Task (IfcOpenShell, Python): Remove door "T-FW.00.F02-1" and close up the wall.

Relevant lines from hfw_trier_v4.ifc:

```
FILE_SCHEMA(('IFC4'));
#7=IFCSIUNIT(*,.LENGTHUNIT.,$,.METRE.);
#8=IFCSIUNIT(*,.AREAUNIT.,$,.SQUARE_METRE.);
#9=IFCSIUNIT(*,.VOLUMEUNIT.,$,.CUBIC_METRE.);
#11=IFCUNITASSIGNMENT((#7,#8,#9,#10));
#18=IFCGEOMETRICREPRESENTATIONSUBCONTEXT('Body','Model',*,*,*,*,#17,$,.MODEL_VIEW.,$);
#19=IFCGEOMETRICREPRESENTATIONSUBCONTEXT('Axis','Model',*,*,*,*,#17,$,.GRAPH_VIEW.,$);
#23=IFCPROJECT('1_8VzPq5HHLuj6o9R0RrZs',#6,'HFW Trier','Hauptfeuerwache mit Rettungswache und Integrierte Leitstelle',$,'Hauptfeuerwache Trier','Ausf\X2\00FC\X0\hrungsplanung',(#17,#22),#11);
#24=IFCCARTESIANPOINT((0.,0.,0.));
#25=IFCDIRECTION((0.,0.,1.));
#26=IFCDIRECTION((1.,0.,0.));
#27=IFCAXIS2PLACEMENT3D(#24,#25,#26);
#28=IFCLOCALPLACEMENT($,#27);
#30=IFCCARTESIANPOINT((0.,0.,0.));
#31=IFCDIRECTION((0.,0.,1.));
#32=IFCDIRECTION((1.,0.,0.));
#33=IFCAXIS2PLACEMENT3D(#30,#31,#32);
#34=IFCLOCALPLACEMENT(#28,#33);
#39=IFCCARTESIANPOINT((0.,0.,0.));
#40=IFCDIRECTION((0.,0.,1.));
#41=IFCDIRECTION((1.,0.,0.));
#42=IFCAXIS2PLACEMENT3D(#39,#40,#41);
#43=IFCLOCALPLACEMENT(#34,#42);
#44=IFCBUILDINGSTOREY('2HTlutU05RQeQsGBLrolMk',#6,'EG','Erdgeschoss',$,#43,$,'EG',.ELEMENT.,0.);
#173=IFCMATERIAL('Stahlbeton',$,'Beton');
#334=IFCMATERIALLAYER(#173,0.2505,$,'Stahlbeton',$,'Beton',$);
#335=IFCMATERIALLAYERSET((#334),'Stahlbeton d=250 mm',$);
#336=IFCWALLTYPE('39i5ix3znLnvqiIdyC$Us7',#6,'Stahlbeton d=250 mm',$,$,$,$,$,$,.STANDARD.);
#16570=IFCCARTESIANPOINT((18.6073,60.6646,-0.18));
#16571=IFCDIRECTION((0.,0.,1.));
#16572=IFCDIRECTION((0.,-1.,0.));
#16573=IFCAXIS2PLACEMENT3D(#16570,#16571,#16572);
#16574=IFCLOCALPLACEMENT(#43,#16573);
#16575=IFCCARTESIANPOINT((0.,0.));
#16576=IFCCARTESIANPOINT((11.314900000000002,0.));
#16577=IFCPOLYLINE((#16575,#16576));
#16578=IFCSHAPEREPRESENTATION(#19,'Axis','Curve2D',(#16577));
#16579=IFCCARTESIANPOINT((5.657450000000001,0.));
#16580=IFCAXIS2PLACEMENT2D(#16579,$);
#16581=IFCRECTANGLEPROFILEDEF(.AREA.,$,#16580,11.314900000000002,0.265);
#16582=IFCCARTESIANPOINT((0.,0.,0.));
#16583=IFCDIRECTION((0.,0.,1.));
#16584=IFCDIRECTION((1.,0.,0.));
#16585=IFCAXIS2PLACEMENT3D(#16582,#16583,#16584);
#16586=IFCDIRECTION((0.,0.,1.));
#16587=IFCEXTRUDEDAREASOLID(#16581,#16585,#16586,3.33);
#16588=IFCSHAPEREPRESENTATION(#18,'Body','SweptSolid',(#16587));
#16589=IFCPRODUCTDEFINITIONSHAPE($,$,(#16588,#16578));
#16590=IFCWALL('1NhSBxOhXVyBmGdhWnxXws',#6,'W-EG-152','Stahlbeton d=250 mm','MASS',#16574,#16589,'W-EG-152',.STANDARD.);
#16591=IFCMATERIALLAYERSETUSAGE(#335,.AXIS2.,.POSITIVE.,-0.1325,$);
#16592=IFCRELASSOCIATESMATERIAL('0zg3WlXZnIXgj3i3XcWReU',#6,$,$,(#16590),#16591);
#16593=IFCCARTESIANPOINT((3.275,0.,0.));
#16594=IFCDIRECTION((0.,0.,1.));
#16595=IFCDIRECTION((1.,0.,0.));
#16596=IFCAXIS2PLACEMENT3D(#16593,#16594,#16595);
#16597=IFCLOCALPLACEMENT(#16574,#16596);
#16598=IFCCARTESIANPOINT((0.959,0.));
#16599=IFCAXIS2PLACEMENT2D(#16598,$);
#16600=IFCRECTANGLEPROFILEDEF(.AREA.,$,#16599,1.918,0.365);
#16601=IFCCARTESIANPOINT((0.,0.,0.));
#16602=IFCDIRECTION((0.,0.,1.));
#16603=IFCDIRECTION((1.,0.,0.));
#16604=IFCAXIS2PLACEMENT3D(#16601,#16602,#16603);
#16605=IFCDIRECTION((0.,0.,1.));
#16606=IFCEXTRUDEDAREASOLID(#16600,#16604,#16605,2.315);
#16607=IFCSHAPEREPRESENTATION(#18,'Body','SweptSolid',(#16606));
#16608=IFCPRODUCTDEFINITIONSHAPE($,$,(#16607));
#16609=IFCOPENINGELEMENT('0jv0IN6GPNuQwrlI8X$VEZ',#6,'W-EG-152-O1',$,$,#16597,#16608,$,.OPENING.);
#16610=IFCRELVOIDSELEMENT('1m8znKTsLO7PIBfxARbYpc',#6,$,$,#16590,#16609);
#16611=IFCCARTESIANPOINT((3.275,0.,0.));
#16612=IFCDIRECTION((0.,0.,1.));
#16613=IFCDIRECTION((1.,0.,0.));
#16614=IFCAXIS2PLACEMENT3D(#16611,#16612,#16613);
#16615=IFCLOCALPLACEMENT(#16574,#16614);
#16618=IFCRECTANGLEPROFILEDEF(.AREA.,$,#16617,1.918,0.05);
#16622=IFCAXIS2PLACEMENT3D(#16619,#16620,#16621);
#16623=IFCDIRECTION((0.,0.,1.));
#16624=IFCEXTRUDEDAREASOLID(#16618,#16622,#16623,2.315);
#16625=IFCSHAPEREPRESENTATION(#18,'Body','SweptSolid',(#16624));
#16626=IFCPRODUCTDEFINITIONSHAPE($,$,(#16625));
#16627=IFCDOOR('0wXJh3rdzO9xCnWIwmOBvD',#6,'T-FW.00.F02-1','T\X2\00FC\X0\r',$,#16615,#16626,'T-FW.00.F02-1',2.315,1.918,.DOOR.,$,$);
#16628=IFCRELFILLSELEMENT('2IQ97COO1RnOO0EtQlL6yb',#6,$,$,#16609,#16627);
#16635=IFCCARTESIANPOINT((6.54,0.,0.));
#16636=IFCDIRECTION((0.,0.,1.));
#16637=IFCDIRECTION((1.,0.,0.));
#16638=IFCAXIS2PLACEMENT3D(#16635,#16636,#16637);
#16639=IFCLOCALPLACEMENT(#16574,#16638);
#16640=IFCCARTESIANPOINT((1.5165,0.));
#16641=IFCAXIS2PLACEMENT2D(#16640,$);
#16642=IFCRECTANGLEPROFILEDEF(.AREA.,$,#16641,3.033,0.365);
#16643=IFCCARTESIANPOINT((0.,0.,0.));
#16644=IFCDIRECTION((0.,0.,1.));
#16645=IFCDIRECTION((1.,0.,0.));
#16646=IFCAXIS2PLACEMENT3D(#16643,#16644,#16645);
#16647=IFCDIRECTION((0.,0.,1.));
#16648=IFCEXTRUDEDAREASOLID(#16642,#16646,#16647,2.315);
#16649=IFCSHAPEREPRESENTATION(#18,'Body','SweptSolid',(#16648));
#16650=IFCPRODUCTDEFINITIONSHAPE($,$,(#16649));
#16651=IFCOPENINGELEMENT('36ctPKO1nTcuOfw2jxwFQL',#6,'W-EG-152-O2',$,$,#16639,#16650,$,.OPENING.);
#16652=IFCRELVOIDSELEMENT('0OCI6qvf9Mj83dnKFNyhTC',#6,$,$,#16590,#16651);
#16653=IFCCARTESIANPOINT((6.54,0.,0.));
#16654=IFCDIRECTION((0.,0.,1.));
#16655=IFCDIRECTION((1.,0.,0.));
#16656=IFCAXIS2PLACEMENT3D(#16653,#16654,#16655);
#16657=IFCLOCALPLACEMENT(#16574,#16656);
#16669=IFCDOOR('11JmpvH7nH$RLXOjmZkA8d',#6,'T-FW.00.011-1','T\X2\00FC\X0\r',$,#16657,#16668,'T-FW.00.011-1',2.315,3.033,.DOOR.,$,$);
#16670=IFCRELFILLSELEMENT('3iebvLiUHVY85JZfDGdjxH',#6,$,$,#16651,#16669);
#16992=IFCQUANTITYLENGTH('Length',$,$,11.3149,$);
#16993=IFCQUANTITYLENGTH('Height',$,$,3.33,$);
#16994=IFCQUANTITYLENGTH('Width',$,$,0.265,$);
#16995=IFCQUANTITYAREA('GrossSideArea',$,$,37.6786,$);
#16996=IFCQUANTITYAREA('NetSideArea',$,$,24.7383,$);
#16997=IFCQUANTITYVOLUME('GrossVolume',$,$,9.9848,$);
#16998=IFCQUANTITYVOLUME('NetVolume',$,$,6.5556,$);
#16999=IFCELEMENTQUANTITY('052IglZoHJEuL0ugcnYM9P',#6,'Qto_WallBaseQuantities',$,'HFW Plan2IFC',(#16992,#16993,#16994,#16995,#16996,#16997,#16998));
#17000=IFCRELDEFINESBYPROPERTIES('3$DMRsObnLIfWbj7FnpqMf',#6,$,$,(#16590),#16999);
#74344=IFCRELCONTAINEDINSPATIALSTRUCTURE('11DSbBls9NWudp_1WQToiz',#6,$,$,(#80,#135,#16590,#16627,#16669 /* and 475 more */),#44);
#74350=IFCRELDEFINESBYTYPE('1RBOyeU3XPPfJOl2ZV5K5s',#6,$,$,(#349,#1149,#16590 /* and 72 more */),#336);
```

```python
import ifcopenshell
import ifcopenshell.api.feature
import ifcopenshell.api.pset
import ifcopenshell.api.root
import ifcopenshell.geom
import ifcopenshell.util.element
import ifcopenshell.util.shape
import ifcopenshell.util.unit

model = ifcopenshell.open("hfw_trier_v4.ifc")
area_scale = ifcopenshell.util.unit.calculate_unit_scale(model, "AREAUNIT")
volume_scale = ifcopenshell.util.unit.calculate_unit_scale(model, "VOLUMEUNIT")
settings = ifcopenshell.geom.settings()


def volume(element):
    """Net volume in cubic metres, openings subtracted."""
    shape = ifcopenshell.geom.create_shape(settings, element)
    return ifcopenshell.util.shape.get_volume(shape.geometry)


door = model.by_guid("0wXJh3rdzO9xCnWIwmOBvD")
opening = door.FillsVoids[0].RelatingOpeningElement
wall = opening.VoidsElements[0].RelatingBuildingElement
before = volume(wall)

ifcopenshell.api.root.remove_product(model, product=door)
ifcopenshell.api.feature.remove_feature(model, feature=opening)

after = volume(wall)
thickness = 0.265  # wall thickness in metres

# Update the wall's stored quantities.
qto = model.by_id(ifcopenshell.util.element.get_pset(wall, "Qto_WallBaseQuantities", should_inherit=False)["id"])
ifcopenshell.api.pset.edit_qto(model, qto=qto, properties={
    "NetSideArea": after / thickness / area_scale,
    "NetVolume": after / volume_scale,
})

print(f"wall volume {before:.3f} -> {after:.3f} m3")

model.write("hfw_trier_v4_rev.ifc")
```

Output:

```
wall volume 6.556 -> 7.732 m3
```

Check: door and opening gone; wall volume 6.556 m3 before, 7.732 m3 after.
